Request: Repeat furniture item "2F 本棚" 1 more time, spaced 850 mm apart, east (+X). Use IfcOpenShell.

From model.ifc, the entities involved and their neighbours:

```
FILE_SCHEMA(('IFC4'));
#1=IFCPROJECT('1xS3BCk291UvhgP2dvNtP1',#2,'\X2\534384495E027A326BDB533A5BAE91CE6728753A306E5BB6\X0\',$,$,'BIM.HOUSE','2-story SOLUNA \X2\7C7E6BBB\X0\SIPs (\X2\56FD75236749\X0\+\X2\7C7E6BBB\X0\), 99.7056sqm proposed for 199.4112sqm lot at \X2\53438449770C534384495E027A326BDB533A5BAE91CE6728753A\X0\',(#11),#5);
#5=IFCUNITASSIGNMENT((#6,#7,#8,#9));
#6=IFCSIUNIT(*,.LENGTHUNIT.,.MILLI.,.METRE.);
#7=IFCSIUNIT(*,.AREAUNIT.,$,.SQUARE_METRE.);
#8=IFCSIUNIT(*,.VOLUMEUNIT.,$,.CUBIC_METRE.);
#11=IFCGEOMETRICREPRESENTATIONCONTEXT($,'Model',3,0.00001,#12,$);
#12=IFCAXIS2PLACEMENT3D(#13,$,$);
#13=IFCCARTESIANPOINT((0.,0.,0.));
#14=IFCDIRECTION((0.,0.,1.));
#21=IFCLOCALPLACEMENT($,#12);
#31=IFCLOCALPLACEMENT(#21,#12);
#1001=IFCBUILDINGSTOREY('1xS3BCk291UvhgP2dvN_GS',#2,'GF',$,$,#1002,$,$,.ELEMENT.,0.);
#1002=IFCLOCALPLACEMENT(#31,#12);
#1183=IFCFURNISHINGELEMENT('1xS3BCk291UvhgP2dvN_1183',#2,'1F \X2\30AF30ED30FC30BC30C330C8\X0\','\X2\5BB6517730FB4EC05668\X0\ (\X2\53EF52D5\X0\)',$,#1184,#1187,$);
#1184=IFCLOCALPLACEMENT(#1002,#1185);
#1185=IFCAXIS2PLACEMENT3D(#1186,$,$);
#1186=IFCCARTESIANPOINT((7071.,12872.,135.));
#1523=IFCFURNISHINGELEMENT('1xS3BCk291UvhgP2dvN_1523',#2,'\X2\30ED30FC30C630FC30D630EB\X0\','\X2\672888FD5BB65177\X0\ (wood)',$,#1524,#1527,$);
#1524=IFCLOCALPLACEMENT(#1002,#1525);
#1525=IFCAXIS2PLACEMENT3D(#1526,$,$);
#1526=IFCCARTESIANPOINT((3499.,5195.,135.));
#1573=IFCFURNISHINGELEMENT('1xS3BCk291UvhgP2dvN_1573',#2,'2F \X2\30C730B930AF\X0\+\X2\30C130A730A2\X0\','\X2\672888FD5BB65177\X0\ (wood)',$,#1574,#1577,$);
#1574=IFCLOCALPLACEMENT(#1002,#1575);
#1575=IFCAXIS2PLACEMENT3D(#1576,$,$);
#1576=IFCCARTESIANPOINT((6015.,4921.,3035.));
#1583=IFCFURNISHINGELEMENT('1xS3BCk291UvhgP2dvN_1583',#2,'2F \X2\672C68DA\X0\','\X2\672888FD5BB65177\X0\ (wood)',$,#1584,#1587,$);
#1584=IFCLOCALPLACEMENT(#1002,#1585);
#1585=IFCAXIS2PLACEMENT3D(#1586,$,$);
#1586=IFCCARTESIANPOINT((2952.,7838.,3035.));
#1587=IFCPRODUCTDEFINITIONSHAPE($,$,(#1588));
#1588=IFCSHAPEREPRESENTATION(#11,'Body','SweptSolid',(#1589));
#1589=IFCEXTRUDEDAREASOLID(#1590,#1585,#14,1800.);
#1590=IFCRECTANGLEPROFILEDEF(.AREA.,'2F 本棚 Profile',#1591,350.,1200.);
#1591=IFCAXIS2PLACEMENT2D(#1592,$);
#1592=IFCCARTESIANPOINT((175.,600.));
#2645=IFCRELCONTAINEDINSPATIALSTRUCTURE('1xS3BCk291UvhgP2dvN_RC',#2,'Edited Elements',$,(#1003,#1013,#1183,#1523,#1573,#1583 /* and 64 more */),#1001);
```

```python
import numpy as np
import ifcopenshell
import ifcopenshell.api.geometry
import ifcopenshell.api.root
import ifcopenshell.util.element
import ifcopenshell.util.placement

model = ifcopenshell.open("model.ifc")


def reuse_history(source, copy):
    """copy_class also copies each property set's owner history, people and application; keep the originals."""
    for rel in copy.IsDefinedBy:
        if rel.is_a("IfcRelDefinesByProperties") and (history := rel.RelatingPropertyDefinition.OwnerHistory):
            rel.RelatingPropertyDefinition.OwnerHistory = source.OwnerHistory
            ifcopenshell.util.element.remove_deep2(model, history)


source = model.by_guid("1xS3BCk291UvhgP2dvN_1583")
base = ifcopenshell.util.placement.get_local_placement(source.ObjectPlacement)
step = np.array([1.0, 0.0, 0.0]) * 850.0

for i in range(1, 2):
    copy = ifcopenshell.api.root.copy_class(model, product=source)
    copy.Representation = ifcopenshell.util.element.copy_deep(
        model, source.Representation, exclude=["IfcGeometricRepresentationContext", "IfcRepresentationMap"]
    )
    reuse_history(source, copy)
    matrix = base.copy()
    matrix[:3, 3] += i * step
    print("added at", matrix[:3, 3].round(3) + 0.0)
    ifcopenshell.api.geometry.edit_object_placement(model, product=copy, matrix=matrix, is_si=False)

model.write("model_rev.ifc")
```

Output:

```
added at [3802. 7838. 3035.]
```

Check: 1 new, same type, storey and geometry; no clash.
